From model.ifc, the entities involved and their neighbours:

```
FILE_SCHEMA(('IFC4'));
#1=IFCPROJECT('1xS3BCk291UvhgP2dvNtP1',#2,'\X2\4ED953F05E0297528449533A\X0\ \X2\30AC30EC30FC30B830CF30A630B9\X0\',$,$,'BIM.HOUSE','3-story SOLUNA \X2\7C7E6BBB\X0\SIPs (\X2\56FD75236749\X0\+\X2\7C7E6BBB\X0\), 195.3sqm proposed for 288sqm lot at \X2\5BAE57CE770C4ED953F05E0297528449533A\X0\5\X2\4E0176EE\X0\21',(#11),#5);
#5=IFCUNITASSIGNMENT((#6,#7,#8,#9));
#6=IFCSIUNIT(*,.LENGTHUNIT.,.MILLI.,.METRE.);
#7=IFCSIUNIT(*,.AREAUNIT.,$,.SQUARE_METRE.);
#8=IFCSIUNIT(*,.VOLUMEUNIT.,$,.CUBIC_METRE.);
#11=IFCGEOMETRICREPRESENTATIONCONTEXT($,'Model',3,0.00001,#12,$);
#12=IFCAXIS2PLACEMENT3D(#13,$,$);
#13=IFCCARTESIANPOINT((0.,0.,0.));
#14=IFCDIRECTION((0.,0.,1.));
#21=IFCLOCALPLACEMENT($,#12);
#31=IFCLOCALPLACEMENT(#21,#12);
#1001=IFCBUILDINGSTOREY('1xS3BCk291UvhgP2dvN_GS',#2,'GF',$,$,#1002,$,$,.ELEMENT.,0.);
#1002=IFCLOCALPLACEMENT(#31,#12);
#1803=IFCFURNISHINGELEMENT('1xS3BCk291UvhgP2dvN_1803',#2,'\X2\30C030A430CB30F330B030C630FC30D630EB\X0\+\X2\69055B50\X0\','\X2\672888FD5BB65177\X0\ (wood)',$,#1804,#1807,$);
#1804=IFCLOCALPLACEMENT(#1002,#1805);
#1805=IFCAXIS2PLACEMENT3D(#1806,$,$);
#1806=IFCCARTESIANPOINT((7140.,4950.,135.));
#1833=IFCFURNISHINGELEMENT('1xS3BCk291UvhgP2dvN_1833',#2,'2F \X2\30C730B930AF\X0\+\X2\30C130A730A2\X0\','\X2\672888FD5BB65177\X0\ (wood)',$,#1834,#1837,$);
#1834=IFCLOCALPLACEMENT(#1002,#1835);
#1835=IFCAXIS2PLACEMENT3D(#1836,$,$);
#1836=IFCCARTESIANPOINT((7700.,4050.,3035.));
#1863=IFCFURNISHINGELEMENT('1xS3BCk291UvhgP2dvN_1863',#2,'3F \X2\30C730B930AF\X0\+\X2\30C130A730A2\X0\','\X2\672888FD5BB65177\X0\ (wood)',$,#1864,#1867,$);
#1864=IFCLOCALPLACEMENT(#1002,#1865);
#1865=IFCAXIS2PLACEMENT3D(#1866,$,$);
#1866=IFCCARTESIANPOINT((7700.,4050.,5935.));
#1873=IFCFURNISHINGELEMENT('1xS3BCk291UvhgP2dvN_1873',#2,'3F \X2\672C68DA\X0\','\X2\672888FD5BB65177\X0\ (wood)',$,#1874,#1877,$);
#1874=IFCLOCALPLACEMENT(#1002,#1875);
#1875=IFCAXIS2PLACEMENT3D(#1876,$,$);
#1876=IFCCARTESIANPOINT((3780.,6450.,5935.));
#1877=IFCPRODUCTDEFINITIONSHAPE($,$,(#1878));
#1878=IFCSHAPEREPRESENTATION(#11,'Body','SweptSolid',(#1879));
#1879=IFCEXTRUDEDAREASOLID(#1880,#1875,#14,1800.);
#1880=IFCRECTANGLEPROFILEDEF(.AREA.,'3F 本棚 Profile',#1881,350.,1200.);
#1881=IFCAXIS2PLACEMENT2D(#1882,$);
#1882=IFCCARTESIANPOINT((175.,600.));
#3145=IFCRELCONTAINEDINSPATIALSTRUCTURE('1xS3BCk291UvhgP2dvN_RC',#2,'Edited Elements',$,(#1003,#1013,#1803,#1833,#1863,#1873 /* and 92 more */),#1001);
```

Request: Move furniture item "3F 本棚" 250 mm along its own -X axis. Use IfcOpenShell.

```python
import ifcopenshell
import ifcopenshell.api.geometry
import ifcopenshell.util.placement
import ifcopenshell.util.unit

model = ifcopenshell.open("model.ifc")
unit_scale = ifcopenshell.util.unit.calculate_unit_scale(model)

item = model.by_id(1873)
matrix = ifcopenshell.util.placement.get_local_placement(item.ObjectPlacement)
matrix[:3, 3] -= matrix[:3, 0] * 0.25 / unit_scale
ifcopenshell.api.geometry.edit_object_placement(model, product=item, matrix=matrix, is_si=False)

print(ifcopenshell.util.placement.get_local_placement(item.ObjectPlacement).round(3) + 0.0)

model.write("model-out.ifc")
```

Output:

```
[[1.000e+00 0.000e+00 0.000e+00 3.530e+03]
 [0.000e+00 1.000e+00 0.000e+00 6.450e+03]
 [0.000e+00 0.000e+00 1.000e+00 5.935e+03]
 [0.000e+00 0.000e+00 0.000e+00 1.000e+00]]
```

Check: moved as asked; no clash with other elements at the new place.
